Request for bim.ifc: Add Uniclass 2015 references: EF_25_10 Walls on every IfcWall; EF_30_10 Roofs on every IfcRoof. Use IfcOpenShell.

First a look at what the model holds.

```python
import ifcopenshell

model = ifcopenshell.open("bim.ifc")
print(model.schema)
print("classifications:", [c.Name for c in model.by_type("IfcClassification")])
for ifc_class in ("IfcDoor", "IfcRoof", "IfcStair", "IfcWall", "IfcWindow"):
    print(ifc_class, len(model.by_type(ifc_class)))
```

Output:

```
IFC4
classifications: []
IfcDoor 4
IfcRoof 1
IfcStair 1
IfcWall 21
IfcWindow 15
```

```python
import ifcopenshell
import ifcopenshell.api.classification

model = ifcopenshell.open("bim.ifc")

system = ifcopenshell.api.classification.add_classification(model, classification="Uniclass 2015")

codes = {
    "IfcWall": ("EF_25_10", "Walls"),
    "IfcRoof": ("EF_30_10", "Roofs"),
}
for ifc_class, (code, name) in codes.items():
    products = model.by_type(ifc_class)
    ifcopenshell.api.classification.add_reference(
        model, products=products, classification=system, identification=code, name=name
    )
    print(code, len(products))

model.write("bim-out.ifc")
```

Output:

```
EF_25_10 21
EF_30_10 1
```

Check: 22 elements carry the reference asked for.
